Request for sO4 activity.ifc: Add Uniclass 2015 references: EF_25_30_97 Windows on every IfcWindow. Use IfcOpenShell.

First a look at what the model holds.

```python
import ifcopenshell

model = ifcopenshell.open("sO4 activity.ifc")
print(model.schema)
print("classifications:", [c.Name for c in model.by_type("IfcClassification")])
for ifc_class in ("IfcDoor", "IfcRoof", "IfcStair", "IfcWall", "IfcWindow"):
    print(ifc_class, len(model.by_type(ifc_class)))
```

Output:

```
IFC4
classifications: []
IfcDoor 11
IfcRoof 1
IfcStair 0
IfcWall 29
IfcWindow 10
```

```python
import ifcopenshell
import ifcopenshell.api.classification

model = ifcopenshell.open("sO4 activity.ifc")

system = ifcopenshell.api.classification.add_classification(model, classification="Uniclass 2015")

codes = {
    "IfcWindow": ("EF_25_30_97", "Windows"),
}
for ifc_class, (code, name) in codes.items():
    products = model.by_type(ifc_class)
    ifcopenshell.api.classification.add_reference(
        model, products=products, classification=system, identification=code, name=name
    )
    print(code, len(products))

model.write("sO4 activity_rev.ifc")
```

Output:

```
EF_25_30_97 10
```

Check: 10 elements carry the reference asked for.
